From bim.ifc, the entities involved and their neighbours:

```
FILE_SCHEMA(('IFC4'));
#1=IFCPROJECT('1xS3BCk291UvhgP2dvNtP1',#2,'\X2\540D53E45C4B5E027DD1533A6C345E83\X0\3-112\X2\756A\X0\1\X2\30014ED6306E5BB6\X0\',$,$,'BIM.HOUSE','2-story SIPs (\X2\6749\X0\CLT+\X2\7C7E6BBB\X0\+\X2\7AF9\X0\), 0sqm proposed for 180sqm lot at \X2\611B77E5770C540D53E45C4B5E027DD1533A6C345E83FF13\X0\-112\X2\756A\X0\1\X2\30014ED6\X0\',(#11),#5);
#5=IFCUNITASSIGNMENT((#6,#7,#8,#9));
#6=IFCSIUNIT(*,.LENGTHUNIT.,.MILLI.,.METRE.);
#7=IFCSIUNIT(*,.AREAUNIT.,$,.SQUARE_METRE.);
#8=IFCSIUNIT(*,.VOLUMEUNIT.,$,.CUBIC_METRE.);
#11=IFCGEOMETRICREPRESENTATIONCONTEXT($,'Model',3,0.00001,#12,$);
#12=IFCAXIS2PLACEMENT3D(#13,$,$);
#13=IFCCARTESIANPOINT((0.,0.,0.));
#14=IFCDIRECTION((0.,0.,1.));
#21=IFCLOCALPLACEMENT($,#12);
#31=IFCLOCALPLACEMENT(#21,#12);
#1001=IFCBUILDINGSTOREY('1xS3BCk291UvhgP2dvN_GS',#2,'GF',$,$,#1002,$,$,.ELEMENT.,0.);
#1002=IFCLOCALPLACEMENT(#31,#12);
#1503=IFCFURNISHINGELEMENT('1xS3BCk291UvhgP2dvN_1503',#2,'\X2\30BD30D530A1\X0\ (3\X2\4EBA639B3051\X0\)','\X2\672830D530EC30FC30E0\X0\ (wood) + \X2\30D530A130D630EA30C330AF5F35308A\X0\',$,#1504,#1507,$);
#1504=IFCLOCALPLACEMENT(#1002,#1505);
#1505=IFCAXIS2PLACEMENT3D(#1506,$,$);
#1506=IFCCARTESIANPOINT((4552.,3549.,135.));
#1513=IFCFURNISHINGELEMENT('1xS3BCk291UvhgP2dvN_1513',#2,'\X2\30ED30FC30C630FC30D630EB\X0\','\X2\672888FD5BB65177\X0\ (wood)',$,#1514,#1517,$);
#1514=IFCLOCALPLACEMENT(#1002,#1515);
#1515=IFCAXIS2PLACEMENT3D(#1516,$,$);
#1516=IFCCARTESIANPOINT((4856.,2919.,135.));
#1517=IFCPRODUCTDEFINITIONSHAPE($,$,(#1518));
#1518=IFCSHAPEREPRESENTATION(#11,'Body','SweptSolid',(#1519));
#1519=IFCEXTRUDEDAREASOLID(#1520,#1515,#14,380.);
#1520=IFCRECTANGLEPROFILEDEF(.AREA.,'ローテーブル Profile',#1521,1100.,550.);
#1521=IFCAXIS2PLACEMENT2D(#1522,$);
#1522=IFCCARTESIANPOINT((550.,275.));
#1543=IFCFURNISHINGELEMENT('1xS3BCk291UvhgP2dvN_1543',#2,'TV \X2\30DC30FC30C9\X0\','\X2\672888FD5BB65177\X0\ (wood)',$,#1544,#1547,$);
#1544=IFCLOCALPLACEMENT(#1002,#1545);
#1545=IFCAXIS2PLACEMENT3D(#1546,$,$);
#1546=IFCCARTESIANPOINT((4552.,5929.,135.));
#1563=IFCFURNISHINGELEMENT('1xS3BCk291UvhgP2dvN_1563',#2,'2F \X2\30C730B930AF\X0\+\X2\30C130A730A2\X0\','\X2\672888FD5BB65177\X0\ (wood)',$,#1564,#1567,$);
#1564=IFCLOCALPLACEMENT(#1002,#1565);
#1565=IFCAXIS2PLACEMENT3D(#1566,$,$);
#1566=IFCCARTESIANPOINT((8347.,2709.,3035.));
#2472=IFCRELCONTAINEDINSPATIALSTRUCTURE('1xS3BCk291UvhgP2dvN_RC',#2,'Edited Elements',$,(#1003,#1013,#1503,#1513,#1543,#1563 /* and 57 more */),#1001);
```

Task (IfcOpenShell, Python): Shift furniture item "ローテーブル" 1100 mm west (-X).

```python
import ifcopenshell
import ifcopenshell.api.geometry
import ifcopenshell.util.placement

model = ifcopenshell.open("bim.ifc")

item = model.by_guid("1xS3BCk291UvhgP2dvN_1513")
matrix = ifcopenshell.util.placement.get_local_placement(item.ObjectPlacement)
matrix[0, 3] -= 1100.0
ifcopenshell.api.geometry.edit_object_placement(model, product=item, matrix=matrix, is_si=False)

print(ifcopenshell.util.placement.get_local_placement(item.ObjectPlacement).round(3) + 0.0)

model.write("bim_rev.ifc")
```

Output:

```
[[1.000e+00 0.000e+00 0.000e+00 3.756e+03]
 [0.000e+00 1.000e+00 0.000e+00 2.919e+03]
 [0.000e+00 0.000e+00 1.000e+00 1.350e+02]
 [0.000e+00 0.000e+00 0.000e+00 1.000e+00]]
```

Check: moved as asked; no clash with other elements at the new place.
